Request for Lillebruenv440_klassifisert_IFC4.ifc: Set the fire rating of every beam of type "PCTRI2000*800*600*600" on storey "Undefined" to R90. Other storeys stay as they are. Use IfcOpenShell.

First a look at what the model holds.

```python
import ifcopenshell
import ifcopenshell.util.element

model = ifcopenshell.open("Lillebruenv440_klassifisert_IFC4.ifc")
print(model.schema)
storey = next(s for s in model.by_type("IfcBuildingStorey") if s.Name == "Undefined")
beams = [e for e in ifcopenshell.util.element.get_decomposition(storey) if e.is_a("IfcBeam")]
seen = {}
for e in beams:
    element_type = ifcopenshell.util.element.get_type(e)
    key = (element_type.Name if element_type != e and element_type else None, ifcopenshell.util.element.get_pset(e, "Pset_BeamCommon", "FireRating"))
    seen[key] = seen.get(key, 0) + 1
for (name, value), count in sorted(seen.items(), key=str):
    print(count, "x", name, "|", value)
```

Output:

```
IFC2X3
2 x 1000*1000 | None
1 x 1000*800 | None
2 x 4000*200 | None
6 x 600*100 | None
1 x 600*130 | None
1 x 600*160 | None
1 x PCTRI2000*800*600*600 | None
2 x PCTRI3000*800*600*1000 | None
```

```python
import ifcopenshell
import ifcopenshell.api.pset
import ifcopenshell.util.element

model = ifcopenshell.open("Lillebruenv440_klassifisert_IFC4.ifc")

storey = next(s for s in model.by_type("IfcBuildingStorey") if s.Name == "Undefined")
beams = [e for e in ifcopenshell.util.element.get_decomposition(storey) if e.is_a("IfcBeam")]

count = 0
for e in beams:
    element_type = ifcopenshell.util.element.get_type(e)
    if element_type in (None, e) or element_type.Name != "PCTRI2000*800*600*600":
        continue
    found = ifcopenshell.util.element.get_pset(e, "Pset_BeamCommon", should_inherit=False)
    if found:
        pset = model.by_id(found["id"])
        if len(ifcopenshell.util.element.get_elements_by_pset(pset)) > 1:
            pset = ifcopenshell.api.pset.unshare_pset(model, products=[e], pset=pset)[0]
    else:
        pset = ifcopenshell.api.pset.add_pset(model, product=e, name="Pset_BeamCommon")
    ifcopenshell.api.pset.edit_pset(model, pset=pset, properties={"FireRating": "R90"})
    count += 1

print(count, "beams updated")

model.write("Lillebruenv440_klassifisert_IFC4_v2.ifc")
```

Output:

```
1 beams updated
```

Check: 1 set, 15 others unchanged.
